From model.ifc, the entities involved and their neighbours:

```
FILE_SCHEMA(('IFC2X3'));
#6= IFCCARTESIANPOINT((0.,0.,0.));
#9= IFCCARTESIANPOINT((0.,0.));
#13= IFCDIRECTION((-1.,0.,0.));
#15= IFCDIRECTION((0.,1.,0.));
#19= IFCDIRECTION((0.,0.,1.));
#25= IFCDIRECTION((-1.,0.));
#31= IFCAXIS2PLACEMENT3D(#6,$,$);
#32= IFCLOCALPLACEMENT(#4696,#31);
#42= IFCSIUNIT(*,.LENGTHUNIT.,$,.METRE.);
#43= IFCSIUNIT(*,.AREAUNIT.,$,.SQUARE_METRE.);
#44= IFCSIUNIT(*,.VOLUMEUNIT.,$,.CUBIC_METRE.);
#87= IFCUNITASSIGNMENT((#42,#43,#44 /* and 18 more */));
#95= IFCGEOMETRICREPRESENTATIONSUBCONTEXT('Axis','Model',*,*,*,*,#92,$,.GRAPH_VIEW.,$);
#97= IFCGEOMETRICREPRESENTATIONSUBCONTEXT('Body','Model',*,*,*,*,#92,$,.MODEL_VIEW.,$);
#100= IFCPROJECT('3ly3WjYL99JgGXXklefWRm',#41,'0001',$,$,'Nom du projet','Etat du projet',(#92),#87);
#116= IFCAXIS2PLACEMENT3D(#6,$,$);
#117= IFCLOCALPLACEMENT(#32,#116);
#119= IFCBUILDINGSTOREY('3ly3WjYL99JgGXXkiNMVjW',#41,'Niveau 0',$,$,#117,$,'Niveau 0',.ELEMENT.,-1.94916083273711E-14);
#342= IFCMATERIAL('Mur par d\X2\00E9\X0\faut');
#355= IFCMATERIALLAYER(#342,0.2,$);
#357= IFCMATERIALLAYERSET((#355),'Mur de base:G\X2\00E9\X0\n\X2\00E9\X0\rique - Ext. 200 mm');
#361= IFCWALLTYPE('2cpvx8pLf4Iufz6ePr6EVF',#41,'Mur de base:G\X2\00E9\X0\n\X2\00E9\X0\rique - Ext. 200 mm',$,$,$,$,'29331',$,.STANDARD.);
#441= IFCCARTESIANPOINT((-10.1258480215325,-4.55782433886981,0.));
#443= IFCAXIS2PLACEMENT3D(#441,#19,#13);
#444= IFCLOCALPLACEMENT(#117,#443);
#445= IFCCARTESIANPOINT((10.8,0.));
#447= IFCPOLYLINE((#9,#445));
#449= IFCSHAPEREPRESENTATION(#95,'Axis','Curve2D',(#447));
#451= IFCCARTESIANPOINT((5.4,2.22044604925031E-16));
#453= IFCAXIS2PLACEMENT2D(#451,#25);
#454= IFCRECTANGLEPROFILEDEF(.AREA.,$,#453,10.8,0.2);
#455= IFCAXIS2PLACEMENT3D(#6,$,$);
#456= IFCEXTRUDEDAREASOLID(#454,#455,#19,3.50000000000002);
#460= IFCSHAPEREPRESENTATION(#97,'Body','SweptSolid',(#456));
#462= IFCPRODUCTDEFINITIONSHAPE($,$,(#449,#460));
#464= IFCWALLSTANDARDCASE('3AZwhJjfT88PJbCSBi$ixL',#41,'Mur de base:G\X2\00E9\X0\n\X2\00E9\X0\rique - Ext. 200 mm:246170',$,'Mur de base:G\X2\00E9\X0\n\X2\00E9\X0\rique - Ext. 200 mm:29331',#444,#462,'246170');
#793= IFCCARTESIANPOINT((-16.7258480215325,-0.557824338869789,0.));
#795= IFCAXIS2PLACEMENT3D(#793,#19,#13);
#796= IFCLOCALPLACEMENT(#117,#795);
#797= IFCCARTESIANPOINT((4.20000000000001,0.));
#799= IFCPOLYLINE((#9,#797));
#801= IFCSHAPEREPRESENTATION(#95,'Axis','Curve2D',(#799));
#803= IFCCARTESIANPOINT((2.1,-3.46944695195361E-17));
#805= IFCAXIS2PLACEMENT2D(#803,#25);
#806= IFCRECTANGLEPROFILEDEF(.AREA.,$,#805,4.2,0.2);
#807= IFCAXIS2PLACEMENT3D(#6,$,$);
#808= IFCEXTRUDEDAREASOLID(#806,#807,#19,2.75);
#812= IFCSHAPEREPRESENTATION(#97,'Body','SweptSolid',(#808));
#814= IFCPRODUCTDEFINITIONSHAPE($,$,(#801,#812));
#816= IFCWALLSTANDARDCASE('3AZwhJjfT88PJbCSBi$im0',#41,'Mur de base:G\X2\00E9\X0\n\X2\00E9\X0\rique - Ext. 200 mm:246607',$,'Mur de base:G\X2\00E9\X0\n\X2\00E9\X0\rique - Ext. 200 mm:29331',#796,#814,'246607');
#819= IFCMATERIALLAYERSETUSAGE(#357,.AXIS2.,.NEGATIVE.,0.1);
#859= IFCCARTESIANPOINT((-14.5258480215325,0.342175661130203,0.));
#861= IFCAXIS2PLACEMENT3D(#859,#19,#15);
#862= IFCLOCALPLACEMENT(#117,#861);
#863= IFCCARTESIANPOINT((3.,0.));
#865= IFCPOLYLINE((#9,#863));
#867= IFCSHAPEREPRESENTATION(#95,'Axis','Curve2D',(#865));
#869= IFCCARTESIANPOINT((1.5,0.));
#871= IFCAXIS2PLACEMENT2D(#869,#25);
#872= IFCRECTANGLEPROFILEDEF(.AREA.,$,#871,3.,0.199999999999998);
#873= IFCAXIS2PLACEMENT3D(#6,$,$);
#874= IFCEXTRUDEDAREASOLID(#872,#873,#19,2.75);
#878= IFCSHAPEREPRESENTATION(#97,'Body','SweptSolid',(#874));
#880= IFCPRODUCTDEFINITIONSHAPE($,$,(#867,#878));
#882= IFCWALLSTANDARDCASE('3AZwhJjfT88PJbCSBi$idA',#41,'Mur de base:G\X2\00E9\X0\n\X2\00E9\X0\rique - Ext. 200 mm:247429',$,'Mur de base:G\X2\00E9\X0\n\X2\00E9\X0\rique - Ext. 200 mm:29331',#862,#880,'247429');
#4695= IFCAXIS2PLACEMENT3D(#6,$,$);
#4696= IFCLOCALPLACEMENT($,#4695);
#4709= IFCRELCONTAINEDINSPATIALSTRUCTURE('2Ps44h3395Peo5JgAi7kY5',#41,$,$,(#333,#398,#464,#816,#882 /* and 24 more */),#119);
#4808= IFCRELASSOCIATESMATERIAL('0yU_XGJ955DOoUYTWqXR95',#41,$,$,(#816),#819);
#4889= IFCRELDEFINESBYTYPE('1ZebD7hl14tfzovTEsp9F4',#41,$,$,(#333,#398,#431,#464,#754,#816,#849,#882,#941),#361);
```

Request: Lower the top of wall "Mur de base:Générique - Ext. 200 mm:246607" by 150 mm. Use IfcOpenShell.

```python
import ifcopenshell
import ifcopenshell.geom
import ifcopenshell.util.representation
import ifcopenshell.util.shape

model = ifcopenshell.open("model.ifc")
settings = ifcopenshell.geom.settings()


def volume(element):
    """Net volume in cubic metres, openings subtracted."""
    shape = ifcopenshell.geom.create_shape(settings, element)
    return ifcopenshell.util.shape.get_volume(shape.geometry)


wall = model.by_guid("3AZwhJjfT88PJbCSBi$im0")
before = volume(wall)

body = ifcopenshell.util.representation.get_representation(wall, "Model", "Body")
solid = body.Items[0]
old_height = solid.Depth
solid.Depth -= 0.15
after = volume(wall)

print(f"height {old_height:g} -> {solid.Depth:g}, volume {before:.3f} -> {after:.3f} m3")

model.write("model-out.ifc")
```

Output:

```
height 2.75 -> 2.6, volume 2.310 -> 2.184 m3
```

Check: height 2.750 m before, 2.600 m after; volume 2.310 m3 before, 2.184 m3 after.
